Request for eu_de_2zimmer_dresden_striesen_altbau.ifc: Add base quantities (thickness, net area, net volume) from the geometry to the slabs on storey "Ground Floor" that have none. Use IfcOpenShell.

First a look at what the model holds.

```python
import ifcopenshell
import ifcopenshell.util.element
import ifcopenshell.util.unit

model = ifcopenshell.open("eu_de_2zimmer_dresden_striesen_altbau.ifc")
print(model.schema)
for unit_type in ("LENGTHUNIT", "AREAUNIT", "VOLUMEUNIT"):
    print(unit_type, ifcopenshell.util.unit.calculate_unit_scale(model, unit_type))
storey = next(s for s in model.by_type("IfcBuildingStorey") if s.Name == "Ground Floor")
slabs = [e for e in ifcopenshell.util.element.get_decomposition(storey) if e.is_a("IfcSlab")]
for e in sorted(slabs, key=lambda e: e.id()):
    print(e.id(), e.is_a(), e.Name, list(ifcopenshell.util.element.get_psets(e, qtos_only=True)), sep=" | ")
```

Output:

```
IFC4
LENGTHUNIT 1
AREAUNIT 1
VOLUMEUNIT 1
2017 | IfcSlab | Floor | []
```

```python
import ifcopenshell
import ifcopenshell.api.pset
import ifcopenshell.geom
import ifcopenshell.util.element
import ifcopenshell.util.shape
import ifcopenshell.util.unit

model = ifcopenshell.open("eu_de_2zimmer_dresden_striesen_altbau.ifc")
unit_scale = ifcopenshell.util.unit.calculate_unit_scale(model)
area_scale = ifcopenshell.util.unit.calculate_unit_scale(model, "AREAUNIT")
volume_scale = ifcopenshell.util.unit.calculate_unit_scale(model, "VOLUMEUNIT")
settings = ifcopenshell.geom.settings()

storey = next(s for s in model.by_type("IfcBuildingStorey") if s.Name == "Ground Floor")
slabs = [e for e in ifcopenshell.util.element.get_decomposition(storey) if e.is_a("IfcSlab")]

for e in sorted(slabs, key=lambda e: e.id()):
    if ifcopenshell.util.element.get_psets(e, qtos_only=True, should_inherit=False):
        continue
    # Geometry comes back in metres, in the element's own axes.
    shape = ifcopenshell.geom.create_shape(settings, e)
    values = {
        "Width": ifcopenshell.util.shape.get_z(shape.geometry) / unit_scale,
        "NetArea": ifcopenshell.util.shape.get_footprint_area(shape.geometry) / area_scale,
        "NetVolume": ifcopenshell.util.shape.get_volume(shape.geometry) / volume_scale,
    }
    qto = ifcopenshell.api.pset.add_qto(model, product=e, name="Qto_SlabBaseQuantities")
    ifcopenshell.api.pset.edit_qto(model, qto=qto, properties=values)
    print(e.id(), {k: round(v, 3) for k, v in values.items()})

model.write("eu_de_2zimmer_dresden_striesen_altbau_updated.ifc")
```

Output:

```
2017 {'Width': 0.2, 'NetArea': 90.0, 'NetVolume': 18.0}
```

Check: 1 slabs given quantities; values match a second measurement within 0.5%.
